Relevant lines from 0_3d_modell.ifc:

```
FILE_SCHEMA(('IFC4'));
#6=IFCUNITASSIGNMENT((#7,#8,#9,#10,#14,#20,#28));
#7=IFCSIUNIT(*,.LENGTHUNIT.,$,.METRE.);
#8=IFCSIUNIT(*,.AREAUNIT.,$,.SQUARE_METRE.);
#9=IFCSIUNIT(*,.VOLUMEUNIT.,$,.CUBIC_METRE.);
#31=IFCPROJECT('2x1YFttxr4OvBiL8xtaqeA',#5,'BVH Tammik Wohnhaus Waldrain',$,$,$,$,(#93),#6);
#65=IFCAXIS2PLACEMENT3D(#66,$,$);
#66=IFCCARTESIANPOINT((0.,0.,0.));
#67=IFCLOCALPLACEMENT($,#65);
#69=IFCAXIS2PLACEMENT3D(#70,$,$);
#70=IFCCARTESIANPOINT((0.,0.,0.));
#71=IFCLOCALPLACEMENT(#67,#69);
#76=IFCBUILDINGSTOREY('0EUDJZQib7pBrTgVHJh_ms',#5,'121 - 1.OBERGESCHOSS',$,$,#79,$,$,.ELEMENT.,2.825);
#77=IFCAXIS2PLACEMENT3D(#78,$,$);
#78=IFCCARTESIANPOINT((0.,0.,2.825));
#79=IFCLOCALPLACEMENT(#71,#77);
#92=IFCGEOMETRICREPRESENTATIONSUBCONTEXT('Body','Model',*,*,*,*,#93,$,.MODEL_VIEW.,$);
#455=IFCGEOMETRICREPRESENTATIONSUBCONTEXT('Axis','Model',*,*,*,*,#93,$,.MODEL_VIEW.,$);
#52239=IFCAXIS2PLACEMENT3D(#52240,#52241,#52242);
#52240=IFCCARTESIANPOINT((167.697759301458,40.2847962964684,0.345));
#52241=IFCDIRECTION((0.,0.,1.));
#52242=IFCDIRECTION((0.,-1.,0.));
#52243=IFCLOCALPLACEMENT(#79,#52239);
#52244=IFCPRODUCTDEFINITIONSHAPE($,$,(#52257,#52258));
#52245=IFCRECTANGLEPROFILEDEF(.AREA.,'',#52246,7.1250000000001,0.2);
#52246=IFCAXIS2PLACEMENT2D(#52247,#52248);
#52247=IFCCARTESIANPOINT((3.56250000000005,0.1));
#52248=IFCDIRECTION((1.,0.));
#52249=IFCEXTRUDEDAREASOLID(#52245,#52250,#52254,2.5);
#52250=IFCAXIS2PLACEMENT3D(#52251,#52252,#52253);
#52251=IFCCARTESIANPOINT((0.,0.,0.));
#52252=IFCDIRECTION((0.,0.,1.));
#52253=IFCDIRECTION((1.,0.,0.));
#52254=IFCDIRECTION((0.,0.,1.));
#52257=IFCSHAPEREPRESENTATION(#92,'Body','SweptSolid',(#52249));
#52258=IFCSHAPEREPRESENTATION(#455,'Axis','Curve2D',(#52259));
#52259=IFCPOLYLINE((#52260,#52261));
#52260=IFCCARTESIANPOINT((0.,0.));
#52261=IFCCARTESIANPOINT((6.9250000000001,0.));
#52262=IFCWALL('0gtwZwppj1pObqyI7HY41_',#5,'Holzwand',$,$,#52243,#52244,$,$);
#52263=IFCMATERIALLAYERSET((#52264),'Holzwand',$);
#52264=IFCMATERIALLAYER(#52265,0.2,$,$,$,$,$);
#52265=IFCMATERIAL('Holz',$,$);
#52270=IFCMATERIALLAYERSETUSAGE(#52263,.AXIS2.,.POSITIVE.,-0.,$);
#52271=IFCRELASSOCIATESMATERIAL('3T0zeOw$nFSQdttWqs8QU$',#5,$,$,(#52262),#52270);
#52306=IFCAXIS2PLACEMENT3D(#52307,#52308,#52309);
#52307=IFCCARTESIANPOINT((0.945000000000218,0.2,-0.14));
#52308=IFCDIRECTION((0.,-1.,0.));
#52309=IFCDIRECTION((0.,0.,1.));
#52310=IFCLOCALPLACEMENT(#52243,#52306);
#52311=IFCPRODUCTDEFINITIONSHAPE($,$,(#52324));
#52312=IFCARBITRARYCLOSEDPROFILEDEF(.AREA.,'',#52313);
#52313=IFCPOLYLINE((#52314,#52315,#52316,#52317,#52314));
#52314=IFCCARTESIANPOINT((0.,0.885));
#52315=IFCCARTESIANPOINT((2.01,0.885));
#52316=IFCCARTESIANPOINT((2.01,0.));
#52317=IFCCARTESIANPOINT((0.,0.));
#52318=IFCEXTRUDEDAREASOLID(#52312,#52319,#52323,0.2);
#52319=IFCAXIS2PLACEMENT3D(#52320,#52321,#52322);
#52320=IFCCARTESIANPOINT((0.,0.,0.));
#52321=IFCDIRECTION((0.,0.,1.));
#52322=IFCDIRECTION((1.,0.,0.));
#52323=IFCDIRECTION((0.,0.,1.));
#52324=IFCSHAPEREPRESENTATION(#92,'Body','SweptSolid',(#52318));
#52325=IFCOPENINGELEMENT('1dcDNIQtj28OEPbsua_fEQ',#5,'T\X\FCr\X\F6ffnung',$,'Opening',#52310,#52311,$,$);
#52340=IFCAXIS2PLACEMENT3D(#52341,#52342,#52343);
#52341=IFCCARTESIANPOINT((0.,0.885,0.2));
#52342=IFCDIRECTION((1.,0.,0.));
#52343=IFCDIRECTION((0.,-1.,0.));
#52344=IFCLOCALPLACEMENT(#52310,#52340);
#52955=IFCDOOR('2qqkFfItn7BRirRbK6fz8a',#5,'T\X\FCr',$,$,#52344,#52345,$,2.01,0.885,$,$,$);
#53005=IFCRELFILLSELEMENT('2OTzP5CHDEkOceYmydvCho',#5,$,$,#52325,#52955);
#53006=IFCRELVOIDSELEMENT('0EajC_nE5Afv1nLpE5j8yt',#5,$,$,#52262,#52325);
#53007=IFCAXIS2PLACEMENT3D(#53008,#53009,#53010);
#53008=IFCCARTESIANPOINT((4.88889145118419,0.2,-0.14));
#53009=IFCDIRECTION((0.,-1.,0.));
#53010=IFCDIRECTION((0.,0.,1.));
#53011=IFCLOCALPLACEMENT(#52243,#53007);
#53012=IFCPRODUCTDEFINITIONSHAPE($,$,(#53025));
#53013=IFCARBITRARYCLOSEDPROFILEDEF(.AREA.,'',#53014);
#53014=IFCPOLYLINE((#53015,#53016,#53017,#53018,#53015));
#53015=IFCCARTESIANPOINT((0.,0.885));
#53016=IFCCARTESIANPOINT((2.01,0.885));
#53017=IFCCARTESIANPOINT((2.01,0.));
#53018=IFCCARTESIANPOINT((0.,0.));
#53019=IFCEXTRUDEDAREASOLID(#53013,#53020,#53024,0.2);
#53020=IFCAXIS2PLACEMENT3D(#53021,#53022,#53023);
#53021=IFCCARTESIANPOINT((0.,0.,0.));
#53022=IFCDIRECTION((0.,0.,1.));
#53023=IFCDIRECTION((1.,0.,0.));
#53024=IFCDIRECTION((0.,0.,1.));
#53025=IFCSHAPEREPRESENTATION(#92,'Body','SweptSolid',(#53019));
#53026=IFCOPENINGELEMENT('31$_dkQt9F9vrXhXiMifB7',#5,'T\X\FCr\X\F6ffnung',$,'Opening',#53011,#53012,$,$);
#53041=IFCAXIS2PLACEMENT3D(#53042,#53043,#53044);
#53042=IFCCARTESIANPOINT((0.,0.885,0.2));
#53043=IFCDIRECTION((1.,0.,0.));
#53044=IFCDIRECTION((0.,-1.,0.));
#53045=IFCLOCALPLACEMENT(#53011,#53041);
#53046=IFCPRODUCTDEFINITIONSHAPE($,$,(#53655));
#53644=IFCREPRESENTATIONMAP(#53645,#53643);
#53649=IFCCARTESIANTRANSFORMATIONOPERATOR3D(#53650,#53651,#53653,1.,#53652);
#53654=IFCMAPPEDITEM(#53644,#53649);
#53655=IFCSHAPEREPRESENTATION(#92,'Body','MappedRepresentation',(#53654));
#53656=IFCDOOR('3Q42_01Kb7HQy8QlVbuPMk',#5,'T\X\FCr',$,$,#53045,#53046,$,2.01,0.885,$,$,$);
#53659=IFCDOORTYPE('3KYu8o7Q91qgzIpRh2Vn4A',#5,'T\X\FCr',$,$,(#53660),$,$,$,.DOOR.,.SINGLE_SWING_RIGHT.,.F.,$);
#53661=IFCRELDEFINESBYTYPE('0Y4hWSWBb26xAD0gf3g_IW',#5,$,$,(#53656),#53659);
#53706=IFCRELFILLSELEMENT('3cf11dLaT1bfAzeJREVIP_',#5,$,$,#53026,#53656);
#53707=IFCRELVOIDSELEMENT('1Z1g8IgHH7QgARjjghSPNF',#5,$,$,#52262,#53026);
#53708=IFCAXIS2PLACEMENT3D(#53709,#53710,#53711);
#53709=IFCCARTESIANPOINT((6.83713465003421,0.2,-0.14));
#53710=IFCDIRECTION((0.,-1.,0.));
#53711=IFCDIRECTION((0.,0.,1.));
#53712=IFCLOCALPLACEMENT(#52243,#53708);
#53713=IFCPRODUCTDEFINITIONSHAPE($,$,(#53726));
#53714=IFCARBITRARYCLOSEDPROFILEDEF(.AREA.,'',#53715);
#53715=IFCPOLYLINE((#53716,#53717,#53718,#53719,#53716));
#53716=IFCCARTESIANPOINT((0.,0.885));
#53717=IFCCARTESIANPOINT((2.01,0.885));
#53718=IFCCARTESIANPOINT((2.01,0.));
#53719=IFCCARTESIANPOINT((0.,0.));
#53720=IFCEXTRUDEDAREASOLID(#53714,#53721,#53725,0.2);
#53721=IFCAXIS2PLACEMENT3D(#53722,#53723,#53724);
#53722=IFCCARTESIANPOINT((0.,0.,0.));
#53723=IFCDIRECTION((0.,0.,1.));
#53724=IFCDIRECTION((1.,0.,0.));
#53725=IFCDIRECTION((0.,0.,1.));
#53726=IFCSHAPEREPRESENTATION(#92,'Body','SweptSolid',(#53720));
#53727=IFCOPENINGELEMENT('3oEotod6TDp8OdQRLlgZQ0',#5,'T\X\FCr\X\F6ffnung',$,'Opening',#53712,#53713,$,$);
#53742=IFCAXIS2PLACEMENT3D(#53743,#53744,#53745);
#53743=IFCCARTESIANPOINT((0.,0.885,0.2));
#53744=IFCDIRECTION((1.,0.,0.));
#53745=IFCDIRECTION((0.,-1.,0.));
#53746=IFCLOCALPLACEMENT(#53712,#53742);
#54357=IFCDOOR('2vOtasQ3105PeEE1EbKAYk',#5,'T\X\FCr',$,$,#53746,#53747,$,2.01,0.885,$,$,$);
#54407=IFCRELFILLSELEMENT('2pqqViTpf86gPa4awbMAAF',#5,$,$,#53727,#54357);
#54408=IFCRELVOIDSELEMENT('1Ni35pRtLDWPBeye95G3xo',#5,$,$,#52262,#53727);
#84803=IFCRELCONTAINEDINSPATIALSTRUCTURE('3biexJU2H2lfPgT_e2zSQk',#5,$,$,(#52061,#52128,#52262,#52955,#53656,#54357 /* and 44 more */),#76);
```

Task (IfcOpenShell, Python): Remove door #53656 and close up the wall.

```python
import ifcopenshell
import ifcopenshell.api.feature
import ifcopenshell.api.root
import ifcopenshell.geom
import ifcopenshell.util.shape

model = ifcopenshell.open("0_3d_modell.ifc")
settings = ifcopenshell.geom.settings()


def volume(element):
    """Net volume in cubic metres, openings subtracted."""
    shape = ifcopenshell.geom.create_shape(settings, element)
    return ifcopenshell.util.shape.get_volume(shape.geometry)


door = model.by_guid("3Q42_01Kb7HQy8QlVbuPMk")
opening = door.FillsVoids[0].RelatingOpeningElement
wall = opening.VoidsElements[0].RelatingBuildingElement
before = volume(wall)

ifcopenshell.api.root.remove_product(model, product=door)
ifcopenshell.api.feature.remove_feature(model, feature=opening)

after = volume(wall)

print(f"wall volume {before:.3f} -> {after:.3f} m3")

model.write("0_3d_modell-out.ifc")
```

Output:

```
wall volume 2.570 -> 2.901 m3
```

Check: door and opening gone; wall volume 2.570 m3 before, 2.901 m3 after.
